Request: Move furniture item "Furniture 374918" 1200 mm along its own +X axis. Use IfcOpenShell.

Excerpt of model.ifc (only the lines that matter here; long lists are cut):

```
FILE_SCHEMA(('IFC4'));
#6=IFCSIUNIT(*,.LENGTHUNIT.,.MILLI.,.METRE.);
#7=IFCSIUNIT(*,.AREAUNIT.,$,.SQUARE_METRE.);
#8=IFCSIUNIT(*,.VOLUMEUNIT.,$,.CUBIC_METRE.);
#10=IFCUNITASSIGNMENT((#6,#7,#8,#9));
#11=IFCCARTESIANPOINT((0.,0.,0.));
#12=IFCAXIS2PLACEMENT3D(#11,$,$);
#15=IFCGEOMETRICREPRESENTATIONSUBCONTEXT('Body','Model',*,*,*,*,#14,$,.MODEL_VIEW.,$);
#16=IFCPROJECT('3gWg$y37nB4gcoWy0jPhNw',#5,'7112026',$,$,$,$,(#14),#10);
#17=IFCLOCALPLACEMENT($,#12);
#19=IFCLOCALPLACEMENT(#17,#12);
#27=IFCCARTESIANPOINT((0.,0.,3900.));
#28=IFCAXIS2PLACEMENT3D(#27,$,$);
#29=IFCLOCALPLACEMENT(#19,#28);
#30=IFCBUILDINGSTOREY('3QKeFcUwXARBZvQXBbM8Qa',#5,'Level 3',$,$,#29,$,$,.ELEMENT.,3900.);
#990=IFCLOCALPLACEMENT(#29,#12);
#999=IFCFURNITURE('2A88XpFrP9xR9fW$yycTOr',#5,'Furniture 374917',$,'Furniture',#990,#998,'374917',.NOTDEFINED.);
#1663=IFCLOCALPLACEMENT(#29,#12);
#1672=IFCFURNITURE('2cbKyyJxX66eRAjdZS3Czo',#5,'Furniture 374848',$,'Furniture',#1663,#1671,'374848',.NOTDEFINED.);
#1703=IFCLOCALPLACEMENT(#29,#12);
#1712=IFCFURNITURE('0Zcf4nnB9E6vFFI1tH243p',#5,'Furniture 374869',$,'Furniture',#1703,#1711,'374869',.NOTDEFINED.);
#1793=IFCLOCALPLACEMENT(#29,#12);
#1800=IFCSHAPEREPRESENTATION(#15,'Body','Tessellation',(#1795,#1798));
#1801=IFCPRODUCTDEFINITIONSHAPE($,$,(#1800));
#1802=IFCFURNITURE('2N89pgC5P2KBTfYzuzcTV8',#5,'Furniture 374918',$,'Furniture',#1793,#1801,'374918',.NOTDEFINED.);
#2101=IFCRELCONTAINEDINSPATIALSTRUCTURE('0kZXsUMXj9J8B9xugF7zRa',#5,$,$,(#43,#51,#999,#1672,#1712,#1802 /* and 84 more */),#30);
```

```python
import ifcopenshell
import ifcopenshell.api.geometry
import ifcopenshell.util.placement
import ifcopenshell.util.unit

model = ifcopenshell.open("model.ifc")
unit_scale = ifcopenshell.util.unit.calculate_unit_scale(model)

item = model.by_guid("2N89pgC5P2KBTfYzuzcTV8")
matrix = ifcopenshell.util.placement.get_local_placement(item.ObjectPlacement)
matrix[:3, 3] += matrix[:3, 0] * 1.2 / unit_scale
ifcopenshell.api.geometry.edit_object_placement(model, product=item, matrix=matrix, is_si=False)

print(ifcopenshell.util.placement.get_local_placement(item.ObjectPlacement).round(3) + 0.0)

model.write("model_edited.ifc")
```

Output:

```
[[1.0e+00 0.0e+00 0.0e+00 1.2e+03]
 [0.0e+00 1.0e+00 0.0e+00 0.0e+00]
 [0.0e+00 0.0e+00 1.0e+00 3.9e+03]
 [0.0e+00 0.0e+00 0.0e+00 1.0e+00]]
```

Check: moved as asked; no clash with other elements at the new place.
